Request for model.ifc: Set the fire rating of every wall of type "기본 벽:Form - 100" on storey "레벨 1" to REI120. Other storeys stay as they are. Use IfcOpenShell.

First a look at what the model holds.

```python
import ifcopenshell
import ifcopenshell.util.element

model = ifcopenshell.open("model.ifc")
print(model.schema)
storey = next(s for s in model.by_type("IfcBuildingStorey") if s.Name == "레벨 1")
walls = [e for e in ifcopenshell.util.element.get_decomposition(storey) if e.is_a("IfcWall")]
seen = {}
for e in walls:
    element_type = ifcopenshell.util.element.get_type(e)
    key = (element_type.Name if element_type != e and element_type else None, ifcopenshell.util.element.get_pset(e, "Pset_WallCommon", "FireRating"))
    seen[key] = seen.get(key, 0) + 1
for (name, value), count in sorted(seen.items(), key=str):
    print(count, "x", name, "|", value)
```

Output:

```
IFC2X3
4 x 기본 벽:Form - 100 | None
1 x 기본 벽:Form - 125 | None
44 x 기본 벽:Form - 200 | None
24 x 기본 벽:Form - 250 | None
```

```python
import ifcopenshell
import ifcopenshell.api.pset
import ifcopenshell.util.element

model = ifcopenshell.open("model.ifc")

storey = next(s for s in model.by_type("IfcBuildingStorey") if s.Name == "레벨 1")
walls = [e for e in ifcopenshell.util.element.get_decomposition(storey) if e.is_a("IfcWall")]

count = 0
for e in walls:
    element_type = ifcopenshell.util.element.get_type(e)
    if element_type in (None, e) or element_type.Name != "기본 벽:Form - 100":
        continue
    # add_pset returns the element's existing set when there is one.
    pset = ifcopenshell.api.pset.add_pset(model, product=e, name="Pset_WallCommon")
    ifcopenshell.api.pset.edit_pset(model, pset=pset, properties={"FireRating": "REI120"})
    count += 1

print(count, "walls updated")

model.write("model_edited.ifc")
```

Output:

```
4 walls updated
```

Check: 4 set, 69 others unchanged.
